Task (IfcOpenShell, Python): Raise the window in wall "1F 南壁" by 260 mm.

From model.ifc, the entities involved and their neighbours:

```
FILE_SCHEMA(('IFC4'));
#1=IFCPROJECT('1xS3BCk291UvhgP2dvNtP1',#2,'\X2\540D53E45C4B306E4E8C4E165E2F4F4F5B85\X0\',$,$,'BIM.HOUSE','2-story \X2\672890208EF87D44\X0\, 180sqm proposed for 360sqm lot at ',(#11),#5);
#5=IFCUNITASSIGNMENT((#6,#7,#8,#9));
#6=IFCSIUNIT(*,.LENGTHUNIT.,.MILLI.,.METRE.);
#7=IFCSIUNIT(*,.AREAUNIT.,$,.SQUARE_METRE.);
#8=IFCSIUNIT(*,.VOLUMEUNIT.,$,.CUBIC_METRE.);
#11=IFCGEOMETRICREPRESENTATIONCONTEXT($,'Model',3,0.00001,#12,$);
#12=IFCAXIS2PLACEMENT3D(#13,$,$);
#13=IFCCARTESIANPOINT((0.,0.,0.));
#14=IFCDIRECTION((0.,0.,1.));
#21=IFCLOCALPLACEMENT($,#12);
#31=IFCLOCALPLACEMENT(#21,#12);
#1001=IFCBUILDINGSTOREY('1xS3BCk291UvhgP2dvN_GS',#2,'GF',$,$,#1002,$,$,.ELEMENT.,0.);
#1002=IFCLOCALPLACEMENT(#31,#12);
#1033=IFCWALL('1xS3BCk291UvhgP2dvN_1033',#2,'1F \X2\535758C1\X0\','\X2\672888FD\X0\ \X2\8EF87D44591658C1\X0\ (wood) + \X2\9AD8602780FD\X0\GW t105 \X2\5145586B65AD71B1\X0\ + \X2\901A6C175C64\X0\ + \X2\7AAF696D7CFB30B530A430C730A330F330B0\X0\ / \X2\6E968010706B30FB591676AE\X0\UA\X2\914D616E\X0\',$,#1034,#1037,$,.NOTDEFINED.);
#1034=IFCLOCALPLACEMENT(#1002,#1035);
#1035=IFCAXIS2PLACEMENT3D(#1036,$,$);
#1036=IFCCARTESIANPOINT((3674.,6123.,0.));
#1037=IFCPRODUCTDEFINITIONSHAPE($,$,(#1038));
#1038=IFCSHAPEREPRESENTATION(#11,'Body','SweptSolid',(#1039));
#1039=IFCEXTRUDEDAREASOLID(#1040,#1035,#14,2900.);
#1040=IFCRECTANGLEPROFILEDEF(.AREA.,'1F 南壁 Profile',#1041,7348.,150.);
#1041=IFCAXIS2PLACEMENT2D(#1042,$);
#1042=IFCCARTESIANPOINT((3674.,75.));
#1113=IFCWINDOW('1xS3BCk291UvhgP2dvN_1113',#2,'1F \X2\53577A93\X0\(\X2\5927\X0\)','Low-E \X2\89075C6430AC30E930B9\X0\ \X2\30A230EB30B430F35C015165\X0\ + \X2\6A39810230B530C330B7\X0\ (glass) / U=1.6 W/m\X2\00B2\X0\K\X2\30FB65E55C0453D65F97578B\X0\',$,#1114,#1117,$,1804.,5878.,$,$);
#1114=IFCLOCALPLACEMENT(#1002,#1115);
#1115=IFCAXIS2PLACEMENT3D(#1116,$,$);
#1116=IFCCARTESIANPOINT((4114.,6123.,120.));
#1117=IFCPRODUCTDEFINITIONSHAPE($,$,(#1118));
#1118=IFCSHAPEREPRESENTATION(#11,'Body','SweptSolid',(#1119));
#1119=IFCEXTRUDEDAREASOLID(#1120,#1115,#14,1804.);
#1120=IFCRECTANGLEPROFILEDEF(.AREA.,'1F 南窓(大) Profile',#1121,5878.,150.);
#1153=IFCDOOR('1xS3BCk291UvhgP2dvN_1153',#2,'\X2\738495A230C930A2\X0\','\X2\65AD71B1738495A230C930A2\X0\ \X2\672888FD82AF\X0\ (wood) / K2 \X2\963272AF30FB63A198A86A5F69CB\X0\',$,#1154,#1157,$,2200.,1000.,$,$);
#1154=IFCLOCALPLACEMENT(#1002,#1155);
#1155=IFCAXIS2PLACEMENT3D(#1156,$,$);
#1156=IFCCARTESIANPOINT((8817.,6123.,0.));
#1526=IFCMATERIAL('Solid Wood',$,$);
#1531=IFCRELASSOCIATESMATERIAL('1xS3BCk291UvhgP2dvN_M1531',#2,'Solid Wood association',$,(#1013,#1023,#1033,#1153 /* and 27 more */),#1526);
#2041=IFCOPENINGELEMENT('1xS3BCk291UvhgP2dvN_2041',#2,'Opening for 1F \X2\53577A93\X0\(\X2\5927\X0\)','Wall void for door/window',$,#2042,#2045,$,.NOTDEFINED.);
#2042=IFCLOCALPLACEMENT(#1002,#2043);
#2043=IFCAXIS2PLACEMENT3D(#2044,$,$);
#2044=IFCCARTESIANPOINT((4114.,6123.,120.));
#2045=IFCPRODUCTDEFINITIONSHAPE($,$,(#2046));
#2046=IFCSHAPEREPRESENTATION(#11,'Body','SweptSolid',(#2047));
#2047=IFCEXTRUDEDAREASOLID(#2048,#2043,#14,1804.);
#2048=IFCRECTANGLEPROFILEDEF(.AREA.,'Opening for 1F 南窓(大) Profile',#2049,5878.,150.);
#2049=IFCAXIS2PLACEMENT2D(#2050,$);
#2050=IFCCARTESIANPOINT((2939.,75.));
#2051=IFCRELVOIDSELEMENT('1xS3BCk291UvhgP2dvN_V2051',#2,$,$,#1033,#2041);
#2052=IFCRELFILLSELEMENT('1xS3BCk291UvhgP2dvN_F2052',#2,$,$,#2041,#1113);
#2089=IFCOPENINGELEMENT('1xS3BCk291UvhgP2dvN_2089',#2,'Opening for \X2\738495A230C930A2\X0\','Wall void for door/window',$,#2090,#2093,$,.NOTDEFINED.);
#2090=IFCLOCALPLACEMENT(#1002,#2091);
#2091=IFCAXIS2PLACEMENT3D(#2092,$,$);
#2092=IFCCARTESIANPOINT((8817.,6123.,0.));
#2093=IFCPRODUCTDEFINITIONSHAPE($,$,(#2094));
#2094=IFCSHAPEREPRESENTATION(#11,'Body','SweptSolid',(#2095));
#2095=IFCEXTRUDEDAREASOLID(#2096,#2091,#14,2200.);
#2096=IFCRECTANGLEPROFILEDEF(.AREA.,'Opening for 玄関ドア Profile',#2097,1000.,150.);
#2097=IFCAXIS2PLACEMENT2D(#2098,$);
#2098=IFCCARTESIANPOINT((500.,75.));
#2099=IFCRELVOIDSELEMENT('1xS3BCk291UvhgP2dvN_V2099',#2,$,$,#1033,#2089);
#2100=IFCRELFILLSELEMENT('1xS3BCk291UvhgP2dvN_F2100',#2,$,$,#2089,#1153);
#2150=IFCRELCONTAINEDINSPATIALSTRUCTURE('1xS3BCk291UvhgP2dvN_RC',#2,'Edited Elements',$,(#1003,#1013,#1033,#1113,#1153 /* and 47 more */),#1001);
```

```python
import numpy as np
import ifcopenshell
import ifcopenshell.api.geometry
import ifcopenshell.util.placement
import ifcopenshell.util.unit

model = ifcopenshell.open("model.ifc")
unit_scale = ifcopenshell.util.unit.calculate_unit_scale(model)

window = model.by_guid("1xS3BCk291UvhgP2dvN_1113")
opening = window.FillsVoids[0].RelatingOpeningElement
dz = 0.26 / unit_scale

shift = np.array([0.0, 0.0, dz])
# The window is not placed relative to its opening, so move both.
for product in (opening, window):
    matrix = ifcopenshell.util.placement.get_local_placement(product.ObjectPlacement)
    matrix[:3, 3] += shift
    ifcopenshell.api.geometry.edit_object_placement(model, product=product, matrix=matrix, is_si=False)

print(f"moved by {dz * unit_scale:+.3f} m")

model.write("model_rev.ifc")
```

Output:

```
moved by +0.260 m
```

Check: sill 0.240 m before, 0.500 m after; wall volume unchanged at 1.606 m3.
